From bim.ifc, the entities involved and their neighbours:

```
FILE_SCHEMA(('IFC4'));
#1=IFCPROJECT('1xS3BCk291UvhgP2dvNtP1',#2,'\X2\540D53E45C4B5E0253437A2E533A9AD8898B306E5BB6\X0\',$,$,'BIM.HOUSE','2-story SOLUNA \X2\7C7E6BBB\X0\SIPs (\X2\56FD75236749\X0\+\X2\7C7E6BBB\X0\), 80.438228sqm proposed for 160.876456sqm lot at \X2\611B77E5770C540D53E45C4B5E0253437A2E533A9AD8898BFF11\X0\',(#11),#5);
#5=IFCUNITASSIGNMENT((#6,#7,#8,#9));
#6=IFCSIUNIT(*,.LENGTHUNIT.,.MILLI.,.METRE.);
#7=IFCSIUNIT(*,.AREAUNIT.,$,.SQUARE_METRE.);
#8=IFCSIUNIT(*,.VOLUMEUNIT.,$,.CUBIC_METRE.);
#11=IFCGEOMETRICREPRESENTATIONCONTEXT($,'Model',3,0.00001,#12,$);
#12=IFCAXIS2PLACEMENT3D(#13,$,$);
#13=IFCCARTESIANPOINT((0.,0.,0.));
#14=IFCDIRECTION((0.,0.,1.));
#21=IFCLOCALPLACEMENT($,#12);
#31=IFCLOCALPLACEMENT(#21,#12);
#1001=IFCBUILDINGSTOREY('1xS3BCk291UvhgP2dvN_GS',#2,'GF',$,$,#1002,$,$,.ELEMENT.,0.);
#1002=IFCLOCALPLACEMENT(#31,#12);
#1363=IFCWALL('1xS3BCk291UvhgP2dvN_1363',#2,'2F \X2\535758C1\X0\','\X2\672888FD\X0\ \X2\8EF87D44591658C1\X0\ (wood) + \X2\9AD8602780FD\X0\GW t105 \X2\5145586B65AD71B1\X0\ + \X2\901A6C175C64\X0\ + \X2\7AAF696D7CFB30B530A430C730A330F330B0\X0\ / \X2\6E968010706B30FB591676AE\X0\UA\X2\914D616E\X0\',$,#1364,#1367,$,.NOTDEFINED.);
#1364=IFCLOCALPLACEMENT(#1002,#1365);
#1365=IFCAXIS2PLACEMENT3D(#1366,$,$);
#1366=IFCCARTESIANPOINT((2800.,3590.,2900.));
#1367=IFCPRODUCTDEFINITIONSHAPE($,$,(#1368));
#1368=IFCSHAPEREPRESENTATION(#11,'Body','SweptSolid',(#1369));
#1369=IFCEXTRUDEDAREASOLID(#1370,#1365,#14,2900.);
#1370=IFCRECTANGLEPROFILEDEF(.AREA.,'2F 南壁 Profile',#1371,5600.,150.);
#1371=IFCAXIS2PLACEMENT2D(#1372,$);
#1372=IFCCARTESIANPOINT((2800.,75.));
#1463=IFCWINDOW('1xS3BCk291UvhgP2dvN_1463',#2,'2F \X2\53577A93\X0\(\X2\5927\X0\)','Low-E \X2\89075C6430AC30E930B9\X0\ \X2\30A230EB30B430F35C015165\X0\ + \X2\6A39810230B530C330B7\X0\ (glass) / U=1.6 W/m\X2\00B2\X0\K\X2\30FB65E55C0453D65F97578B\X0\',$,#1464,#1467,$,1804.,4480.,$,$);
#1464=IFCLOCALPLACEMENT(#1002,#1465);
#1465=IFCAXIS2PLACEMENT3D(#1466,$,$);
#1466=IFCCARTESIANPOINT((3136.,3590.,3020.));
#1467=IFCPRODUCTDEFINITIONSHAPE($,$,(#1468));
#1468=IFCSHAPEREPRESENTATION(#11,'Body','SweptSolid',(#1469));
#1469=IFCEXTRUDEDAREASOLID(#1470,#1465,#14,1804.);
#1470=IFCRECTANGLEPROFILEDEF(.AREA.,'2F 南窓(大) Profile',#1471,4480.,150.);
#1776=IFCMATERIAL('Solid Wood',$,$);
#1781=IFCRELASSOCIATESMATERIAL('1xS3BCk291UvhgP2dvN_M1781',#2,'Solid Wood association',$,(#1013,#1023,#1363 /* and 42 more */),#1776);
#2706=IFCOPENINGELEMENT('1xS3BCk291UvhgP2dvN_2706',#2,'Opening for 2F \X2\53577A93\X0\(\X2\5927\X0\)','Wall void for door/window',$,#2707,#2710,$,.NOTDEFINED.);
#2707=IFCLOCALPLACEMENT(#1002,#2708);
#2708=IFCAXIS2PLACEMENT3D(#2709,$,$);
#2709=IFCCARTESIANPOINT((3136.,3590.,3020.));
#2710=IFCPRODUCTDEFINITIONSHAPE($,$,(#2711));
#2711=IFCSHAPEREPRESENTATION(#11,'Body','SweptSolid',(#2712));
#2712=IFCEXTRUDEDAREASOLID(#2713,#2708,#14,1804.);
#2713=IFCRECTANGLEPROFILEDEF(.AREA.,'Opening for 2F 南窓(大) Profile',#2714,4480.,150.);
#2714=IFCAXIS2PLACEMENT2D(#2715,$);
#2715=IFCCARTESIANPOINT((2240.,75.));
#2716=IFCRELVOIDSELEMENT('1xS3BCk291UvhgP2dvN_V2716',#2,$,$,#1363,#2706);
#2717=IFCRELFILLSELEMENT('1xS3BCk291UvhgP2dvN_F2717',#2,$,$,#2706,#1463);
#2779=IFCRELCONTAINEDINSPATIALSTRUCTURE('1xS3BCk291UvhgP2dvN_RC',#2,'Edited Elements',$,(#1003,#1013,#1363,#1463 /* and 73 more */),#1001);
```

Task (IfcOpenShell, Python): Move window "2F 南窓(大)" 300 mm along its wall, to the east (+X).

```python
import ifcopenshell
import ifcopenshell.api.geometry
import ifcopenshell.util.placement

model = ifcopenshell.open("bim.ifc")

window = model.by_id(1463)
opening = window.FillsVoids[0].RelatingOpeningElement
wall = opening.VoidsElements[0].RelatingBuildingElement

wall_matrix = ifcopenshell.util.placement.get_local_placement(wall.ObjectPlacement)
shift = wall_matrix[:3, 0] * 300.0
before = ifcopenshell.util.placement.get_local_placement(window.ObjectPlacement)[:3, 3].copy()

# The window is not placed relative to its opening, so move both.
for product in (opening, window):
    matrix = ifcopenshell.util.placement.get_local_placement(product.ObjectPlacement)
    matrix[:3, 3] += shift
    ifcopenshell.api.geometry.edit_object_placement(model, product=product, matrix=matrix, is_si=False)

after = ifcopenshell.util.placement.get_local_placement(window.ObjectPlacement)[:3, 3]
print("window moved by", (after - before).round(3) + 0.0)

model.write("bim_rev.ifc")
```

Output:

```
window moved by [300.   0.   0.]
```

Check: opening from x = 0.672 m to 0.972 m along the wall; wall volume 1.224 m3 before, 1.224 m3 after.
